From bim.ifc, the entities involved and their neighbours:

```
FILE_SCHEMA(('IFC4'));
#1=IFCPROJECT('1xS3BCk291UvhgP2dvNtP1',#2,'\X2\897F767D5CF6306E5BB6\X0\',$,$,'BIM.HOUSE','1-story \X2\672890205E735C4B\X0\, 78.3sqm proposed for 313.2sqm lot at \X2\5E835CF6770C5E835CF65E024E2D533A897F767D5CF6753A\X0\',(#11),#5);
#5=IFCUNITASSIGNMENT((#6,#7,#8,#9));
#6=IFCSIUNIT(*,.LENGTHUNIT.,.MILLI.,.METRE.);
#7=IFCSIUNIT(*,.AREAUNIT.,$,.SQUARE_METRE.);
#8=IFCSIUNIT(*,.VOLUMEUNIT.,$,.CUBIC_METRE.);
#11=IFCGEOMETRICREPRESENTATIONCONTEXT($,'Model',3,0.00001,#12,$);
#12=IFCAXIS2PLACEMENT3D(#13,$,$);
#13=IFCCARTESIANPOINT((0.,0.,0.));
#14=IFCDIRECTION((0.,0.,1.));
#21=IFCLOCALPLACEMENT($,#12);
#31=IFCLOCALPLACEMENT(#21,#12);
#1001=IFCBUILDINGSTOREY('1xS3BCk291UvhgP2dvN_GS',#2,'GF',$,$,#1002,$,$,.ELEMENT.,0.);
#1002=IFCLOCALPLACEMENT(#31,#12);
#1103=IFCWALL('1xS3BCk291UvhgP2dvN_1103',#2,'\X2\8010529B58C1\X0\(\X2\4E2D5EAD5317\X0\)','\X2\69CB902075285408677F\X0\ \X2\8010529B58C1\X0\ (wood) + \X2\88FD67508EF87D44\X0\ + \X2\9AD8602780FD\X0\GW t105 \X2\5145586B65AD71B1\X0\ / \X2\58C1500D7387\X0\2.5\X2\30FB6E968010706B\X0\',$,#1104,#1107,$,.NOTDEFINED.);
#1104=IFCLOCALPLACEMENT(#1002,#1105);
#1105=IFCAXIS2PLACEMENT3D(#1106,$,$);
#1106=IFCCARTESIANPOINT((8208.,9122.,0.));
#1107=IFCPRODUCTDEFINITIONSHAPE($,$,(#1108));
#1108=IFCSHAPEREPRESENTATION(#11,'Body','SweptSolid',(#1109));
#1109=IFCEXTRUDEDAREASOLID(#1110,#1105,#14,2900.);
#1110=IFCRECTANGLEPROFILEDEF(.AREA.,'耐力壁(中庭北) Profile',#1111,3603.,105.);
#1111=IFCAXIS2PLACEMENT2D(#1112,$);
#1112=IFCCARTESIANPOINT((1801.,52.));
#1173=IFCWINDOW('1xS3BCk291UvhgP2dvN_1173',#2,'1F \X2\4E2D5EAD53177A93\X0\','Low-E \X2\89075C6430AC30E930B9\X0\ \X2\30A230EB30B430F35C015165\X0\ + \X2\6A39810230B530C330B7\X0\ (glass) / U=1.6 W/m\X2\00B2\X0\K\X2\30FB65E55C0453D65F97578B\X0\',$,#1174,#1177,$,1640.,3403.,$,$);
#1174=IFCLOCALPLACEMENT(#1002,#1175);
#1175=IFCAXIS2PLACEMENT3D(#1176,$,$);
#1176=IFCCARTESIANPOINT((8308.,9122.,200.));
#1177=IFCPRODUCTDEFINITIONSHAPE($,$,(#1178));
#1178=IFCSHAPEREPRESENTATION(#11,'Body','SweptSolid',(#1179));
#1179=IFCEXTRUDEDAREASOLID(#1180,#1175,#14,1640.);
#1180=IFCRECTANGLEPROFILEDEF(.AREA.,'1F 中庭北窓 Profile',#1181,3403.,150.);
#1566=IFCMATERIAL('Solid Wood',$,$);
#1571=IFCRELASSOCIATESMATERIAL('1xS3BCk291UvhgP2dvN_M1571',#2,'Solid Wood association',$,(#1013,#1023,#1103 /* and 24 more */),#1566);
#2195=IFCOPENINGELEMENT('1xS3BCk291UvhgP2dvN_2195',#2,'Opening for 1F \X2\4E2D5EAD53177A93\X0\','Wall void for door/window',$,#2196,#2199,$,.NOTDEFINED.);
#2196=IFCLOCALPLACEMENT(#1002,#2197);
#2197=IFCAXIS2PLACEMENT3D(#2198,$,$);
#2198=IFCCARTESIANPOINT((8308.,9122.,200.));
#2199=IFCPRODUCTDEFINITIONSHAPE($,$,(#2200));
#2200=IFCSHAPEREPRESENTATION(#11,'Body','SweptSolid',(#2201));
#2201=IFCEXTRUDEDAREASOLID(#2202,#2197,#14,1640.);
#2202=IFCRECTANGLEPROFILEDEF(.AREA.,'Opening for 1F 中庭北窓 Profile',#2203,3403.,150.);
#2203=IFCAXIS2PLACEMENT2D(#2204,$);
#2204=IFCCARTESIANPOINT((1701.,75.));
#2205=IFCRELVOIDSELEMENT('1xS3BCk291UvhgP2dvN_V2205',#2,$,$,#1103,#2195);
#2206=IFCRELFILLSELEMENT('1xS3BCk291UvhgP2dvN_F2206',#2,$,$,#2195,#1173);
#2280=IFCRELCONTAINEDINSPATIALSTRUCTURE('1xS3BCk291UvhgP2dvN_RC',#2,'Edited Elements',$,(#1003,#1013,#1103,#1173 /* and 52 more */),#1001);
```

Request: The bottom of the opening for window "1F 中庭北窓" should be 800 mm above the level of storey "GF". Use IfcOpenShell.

```python
import numpy as np
import ifcopenshell
import ifcopenshell.api.geometry
import ifcopenshell.geom
import ifcopenshell.util.element
import ifcopenshell.util.placement
import ifcopenshell.util.shape
import ifcopenshell.util.unit

model = ifcopenshell.open("bim.ifc")
unit_scale = ifcopenshell.util.unit.calculate_unit_scale(model)

window = model.by_guid("1xS3BCk291UvhgP2dvN_1173")
opening = window.FillsVoids[0].RelatingOpeningElement
storey = ifcopenshell.util.element.get_container(window, ifc_class="IfcBuildingStorey")
level = ifcopenshell.util.placement.get_local_placement(storey.ObjectPlacement)[2, 3]

# The opening's origin need not be at the sill, so measure its lowest point.
shape = ifcopenshell.geom.create_shape(ifcopenshell.geom.settings(), opening)
bottom = ifcopenshell.util.shape.get_shape_bottom_elevation(shape, shape.geometry) / unit_scale
dz = level + 0.8 / unit_scale - bottom

shift = np.array([0.0, 0.0, dz])
# The window is not placed relative to its opening, so move both.
for product in (opening, window):
    matrix = ifcopenshell.util.placement.get_local_placement(product.ObjectPlacement)
    matrix[:3, 3] += shift
    ifcopenshell.api.geometry.edit_object_placement(model, product=product, matrix=matrix, is_si=False)

print(f"moved by {dz * unit_scale:+.3f} m")

model.write("bim_rev.ifc")
```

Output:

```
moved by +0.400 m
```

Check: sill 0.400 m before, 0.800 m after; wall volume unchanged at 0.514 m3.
